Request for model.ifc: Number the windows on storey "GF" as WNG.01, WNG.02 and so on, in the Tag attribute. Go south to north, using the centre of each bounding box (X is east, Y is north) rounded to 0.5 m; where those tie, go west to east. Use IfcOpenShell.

First a look at what the model holds.

```python
import ifcopenshell
import ifcopenshell.util.element
import ifcopenshell.util.placement

model = ifcopenshell.open("model.ifc")
print(model.schema)
storey = next(s for s in model.by_type("IfcBuildingStorey") if s.Name == "GF")
windows = [e for e in ifcopenshell.util.element.get_decomposition(storey) if e.is_a("IfcWindow")]
for e in sorted(windows, key=lambda e: e.id()):
    origin = ifcopenshell.util.placement.get_local_placement(e.ObjectPlacement)[:3, 3]
    print(e.id(), e.Tag, e.Name, origin.round(2) + 0.0, sep=" | ")
```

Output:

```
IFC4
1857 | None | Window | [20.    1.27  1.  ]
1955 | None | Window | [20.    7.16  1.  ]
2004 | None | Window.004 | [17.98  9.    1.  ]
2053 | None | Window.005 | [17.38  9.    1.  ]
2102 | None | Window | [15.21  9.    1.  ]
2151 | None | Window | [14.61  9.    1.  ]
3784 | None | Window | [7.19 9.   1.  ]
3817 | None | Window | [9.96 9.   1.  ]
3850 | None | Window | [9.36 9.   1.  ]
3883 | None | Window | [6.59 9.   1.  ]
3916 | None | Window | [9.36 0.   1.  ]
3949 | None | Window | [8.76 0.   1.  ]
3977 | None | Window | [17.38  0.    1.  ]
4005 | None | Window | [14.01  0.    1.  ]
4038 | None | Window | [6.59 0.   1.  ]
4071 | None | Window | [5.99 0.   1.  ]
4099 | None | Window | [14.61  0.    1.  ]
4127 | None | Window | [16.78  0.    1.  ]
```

```python
import ifcopenshell
import ifcopenshell.geom
import ifcopenshell.util.element
import ifcopenshell.util.shape

model = ifcopenshell.open("model.ifc")
settings = ifcopenshell.geom.settings()
settings.set("use-world-coords", True)


def centre(element):
    shape = ifcopenshell.geom.create_shape(settings, element)
    return ifcopenshell.util.shape.get_bbox_centroid(shape.geometry)


storey = next(s for s in model.by_type("IfcBuildingStorey") if s.Name == "GF")
windows = [e for e in ifcopenshell.util.element.get_decomposition(storey) if e.is_a("IfcWindow")]

# Insertion points can sit at a corner or the storey origin, so sort by the geometry (in metres).
centres = {e: centre(e) for e in windows}
windows.sort(key=lambda e: (round(centres[e][1] / 0.5), centres[e][0]))

for i, e in enumerate(windows, start=1):
    number = f"WNG.{i:02d}"
    e.Tag = number
    print(e.id(), number)

model.write("model_v2.ifc")
```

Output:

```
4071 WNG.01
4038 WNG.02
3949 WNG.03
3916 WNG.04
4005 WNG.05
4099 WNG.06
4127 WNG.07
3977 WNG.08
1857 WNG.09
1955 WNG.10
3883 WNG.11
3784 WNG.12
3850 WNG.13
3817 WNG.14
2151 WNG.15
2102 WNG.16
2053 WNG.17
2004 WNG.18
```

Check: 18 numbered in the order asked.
